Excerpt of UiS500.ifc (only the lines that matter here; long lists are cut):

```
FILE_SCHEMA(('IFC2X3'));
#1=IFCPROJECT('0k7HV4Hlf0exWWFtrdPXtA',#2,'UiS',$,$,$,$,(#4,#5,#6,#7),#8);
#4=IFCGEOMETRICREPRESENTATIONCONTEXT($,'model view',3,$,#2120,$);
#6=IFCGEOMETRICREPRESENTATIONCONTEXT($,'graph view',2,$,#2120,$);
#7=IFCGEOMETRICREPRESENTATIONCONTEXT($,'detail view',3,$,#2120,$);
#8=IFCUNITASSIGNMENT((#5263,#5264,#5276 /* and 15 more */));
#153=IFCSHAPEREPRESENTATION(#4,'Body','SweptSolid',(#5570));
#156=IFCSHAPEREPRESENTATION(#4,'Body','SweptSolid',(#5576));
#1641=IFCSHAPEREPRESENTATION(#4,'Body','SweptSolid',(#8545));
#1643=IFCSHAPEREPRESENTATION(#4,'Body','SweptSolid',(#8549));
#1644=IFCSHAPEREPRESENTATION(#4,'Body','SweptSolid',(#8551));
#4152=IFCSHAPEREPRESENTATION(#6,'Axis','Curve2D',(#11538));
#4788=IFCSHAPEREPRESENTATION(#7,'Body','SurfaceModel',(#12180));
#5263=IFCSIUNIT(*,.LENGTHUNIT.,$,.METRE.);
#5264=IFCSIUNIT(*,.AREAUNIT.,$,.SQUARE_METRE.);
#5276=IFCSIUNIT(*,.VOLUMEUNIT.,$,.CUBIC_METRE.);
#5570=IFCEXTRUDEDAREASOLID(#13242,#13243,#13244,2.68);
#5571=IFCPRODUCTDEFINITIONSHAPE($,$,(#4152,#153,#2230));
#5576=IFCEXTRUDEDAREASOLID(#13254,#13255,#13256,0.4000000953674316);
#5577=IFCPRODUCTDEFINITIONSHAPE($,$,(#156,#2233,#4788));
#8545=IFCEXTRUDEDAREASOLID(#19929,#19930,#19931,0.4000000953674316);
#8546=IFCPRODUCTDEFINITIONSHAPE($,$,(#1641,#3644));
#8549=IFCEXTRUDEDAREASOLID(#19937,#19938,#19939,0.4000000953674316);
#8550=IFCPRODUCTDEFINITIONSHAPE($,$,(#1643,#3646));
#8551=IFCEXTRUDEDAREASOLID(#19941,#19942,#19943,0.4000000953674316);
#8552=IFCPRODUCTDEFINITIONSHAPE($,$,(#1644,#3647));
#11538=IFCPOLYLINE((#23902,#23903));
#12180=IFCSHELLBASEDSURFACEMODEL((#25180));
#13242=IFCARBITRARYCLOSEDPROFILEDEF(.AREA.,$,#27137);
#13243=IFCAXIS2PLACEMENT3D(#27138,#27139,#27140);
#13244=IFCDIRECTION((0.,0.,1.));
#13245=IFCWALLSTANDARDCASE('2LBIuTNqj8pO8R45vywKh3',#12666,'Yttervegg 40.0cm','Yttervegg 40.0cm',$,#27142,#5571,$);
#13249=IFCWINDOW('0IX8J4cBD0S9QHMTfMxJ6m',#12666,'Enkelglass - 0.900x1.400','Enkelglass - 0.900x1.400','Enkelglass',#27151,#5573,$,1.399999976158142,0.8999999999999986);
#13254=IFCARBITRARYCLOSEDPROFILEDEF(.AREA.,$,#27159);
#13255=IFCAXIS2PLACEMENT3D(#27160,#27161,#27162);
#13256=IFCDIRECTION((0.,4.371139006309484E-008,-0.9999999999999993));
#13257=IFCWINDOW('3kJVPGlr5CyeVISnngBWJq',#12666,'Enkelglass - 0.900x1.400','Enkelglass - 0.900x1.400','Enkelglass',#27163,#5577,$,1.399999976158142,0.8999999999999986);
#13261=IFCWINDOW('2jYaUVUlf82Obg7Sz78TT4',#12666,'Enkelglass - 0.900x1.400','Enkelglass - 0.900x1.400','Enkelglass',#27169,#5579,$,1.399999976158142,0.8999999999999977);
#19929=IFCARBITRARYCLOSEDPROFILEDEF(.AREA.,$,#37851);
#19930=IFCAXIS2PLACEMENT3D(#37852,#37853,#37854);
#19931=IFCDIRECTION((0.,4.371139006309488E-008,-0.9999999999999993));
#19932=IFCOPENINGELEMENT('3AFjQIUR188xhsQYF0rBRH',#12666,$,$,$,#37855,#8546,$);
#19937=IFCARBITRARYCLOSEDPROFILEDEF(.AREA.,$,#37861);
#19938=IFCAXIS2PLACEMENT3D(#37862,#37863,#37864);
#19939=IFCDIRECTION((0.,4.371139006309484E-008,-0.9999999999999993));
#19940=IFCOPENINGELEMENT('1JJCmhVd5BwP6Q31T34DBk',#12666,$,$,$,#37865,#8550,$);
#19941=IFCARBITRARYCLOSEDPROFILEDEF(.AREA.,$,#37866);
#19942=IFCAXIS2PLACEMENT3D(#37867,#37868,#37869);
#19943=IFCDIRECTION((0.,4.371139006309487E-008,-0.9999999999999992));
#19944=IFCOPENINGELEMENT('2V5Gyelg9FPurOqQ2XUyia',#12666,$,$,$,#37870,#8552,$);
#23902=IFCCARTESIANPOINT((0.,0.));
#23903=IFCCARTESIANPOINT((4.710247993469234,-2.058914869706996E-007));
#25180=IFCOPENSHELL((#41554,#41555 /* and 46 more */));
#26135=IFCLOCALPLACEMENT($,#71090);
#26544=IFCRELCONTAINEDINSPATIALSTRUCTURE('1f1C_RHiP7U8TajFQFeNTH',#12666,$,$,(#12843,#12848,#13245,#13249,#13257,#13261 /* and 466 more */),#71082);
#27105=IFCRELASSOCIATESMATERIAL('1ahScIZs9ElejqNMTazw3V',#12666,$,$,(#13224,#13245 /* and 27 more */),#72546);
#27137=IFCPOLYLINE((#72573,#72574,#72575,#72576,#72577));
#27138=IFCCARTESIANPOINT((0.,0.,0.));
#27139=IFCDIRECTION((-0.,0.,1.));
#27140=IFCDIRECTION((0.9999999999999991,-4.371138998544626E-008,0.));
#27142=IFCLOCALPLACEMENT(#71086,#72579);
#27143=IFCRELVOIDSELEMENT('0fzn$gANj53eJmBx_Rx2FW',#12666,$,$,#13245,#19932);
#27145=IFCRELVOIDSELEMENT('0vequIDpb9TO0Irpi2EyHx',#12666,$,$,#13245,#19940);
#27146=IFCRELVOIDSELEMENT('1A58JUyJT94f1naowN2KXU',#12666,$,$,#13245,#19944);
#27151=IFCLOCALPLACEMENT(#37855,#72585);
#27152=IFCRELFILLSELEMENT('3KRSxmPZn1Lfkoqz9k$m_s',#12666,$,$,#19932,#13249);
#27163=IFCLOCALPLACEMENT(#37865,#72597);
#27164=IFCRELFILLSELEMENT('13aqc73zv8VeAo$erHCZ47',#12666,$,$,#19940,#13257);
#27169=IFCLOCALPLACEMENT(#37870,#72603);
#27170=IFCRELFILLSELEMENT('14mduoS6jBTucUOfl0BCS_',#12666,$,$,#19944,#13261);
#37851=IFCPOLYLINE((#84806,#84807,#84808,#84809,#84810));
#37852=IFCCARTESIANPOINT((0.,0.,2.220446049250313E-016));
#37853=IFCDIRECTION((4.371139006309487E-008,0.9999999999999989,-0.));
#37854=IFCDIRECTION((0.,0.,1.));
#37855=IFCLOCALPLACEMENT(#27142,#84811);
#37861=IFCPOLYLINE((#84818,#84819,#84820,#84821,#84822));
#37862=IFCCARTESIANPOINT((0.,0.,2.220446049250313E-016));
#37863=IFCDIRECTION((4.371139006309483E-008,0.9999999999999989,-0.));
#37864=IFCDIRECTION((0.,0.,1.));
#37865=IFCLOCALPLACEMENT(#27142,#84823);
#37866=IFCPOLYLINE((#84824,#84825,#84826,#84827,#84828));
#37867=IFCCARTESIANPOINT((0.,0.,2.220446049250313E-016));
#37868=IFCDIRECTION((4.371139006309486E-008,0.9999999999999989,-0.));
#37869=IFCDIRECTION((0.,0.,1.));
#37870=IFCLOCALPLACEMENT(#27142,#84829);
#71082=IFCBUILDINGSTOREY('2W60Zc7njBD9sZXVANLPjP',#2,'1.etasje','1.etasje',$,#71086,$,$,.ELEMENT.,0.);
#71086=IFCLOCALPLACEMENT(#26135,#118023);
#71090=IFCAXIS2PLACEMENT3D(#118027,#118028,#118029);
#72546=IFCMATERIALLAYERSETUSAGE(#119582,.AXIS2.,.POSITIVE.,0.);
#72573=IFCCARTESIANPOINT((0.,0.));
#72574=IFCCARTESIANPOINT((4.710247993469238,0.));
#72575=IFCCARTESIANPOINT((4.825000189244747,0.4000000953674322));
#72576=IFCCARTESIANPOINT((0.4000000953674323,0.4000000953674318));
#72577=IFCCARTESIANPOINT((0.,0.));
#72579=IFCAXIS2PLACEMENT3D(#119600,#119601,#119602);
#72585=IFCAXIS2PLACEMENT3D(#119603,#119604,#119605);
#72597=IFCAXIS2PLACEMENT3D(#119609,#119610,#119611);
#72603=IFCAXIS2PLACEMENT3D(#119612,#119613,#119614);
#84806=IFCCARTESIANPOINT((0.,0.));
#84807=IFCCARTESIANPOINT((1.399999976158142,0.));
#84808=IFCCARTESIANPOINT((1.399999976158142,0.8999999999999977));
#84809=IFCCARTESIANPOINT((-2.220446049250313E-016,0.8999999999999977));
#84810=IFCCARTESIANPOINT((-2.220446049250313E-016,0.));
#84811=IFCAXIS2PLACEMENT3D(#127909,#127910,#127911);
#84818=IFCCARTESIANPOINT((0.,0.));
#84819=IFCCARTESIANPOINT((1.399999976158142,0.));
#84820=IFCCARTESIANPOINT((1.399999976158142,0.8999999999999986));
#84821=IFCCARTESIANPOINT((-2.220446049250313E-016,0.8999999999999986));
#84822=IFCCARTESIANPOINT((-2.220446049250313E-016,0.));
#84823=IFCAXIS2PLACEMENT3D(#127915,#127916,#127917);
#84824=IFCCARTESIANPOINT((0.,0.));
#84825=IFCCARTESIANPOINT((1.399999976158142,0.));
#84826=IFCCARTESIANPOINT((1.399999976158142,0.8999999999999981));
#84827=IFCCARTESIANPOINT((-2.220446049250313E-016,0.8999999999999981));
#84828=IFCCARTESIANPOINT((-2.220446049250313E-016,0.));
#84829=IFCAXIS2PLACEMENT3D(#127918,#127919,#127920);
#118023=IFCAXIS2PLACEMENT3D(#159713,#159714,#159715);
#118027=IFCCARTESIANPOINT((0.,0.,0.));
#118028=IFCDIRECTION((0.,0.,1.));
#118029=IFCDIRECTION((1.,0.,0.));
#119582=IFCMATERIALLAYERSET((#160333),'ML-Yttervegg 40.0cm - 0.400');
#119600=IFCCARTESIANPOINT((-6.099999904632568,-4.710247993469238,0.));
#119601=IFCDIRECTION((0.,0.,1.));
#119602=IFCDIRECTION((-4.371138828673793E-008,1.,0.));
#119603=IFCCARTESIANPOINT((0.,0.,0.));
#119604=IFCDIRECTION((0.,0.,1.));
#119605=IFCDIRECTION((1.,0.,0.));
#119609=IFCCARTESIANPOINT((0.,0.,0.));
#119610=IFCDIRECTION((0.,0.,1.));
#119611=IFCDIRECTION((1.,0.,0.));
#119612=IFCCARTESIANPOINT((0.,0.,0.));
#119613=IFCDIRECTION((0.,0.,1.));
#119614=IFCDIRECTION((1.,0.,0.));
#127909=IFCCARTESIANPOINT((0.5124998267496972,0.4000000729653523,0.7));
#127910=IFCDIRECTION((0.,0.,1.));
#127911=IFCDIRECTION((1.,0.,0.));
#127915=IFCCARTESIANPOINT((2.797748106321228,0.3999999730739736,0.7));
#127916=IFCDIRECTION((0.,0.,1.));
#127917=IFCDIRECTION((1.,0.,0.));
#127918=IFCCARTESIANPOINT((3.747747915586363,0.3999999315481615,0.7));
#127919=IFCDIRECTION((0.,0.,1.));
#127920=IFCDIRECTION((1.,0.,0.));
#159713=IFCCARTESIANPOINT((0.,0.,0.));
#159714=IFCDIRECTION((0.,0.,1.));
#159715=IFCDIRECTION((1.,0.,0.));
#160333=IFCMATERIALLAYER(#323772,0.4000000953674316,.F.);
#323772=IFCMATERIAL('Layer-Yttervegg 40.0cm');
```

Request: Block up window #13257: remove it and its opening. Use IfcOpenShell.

```python
import ifcopenshell
import ifcopenshell.api.feature
import ifcopenshell.api.root
import ifcopenshell.geom
import ifcopenshell.util.shape

model = ifcopenshell.open("UiS500.ifc")
settings = ifcopenshell.geom.settings()


def volume(element):
    """Net volume in cubic metres, openings subtracted."""
    shape = ifcopenshell.geom.create_shape(settings, element)
    return ifcopenshell.util.shape.get_volume(shape.geometry)


window = model.by_id(13257)
opening = window.FillsVoids[0].RelatingOpeningElement
wall = opening.VoidsElements[0].RelatingBuildingElement
before = volume(wall)

ifcopenshell.api.root.remove_product(model, product=window)
ifcopenshell.api.feature.remove_feature(model, feature=opening)

after = volume(wall)

print(f"wall volume {before:.3f} -> {after:.3f} m3")

model.write("UiS500_updated.ifc")
```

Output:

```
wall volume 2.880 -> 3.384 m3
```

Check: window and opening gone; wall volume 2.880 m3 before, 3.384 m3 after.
